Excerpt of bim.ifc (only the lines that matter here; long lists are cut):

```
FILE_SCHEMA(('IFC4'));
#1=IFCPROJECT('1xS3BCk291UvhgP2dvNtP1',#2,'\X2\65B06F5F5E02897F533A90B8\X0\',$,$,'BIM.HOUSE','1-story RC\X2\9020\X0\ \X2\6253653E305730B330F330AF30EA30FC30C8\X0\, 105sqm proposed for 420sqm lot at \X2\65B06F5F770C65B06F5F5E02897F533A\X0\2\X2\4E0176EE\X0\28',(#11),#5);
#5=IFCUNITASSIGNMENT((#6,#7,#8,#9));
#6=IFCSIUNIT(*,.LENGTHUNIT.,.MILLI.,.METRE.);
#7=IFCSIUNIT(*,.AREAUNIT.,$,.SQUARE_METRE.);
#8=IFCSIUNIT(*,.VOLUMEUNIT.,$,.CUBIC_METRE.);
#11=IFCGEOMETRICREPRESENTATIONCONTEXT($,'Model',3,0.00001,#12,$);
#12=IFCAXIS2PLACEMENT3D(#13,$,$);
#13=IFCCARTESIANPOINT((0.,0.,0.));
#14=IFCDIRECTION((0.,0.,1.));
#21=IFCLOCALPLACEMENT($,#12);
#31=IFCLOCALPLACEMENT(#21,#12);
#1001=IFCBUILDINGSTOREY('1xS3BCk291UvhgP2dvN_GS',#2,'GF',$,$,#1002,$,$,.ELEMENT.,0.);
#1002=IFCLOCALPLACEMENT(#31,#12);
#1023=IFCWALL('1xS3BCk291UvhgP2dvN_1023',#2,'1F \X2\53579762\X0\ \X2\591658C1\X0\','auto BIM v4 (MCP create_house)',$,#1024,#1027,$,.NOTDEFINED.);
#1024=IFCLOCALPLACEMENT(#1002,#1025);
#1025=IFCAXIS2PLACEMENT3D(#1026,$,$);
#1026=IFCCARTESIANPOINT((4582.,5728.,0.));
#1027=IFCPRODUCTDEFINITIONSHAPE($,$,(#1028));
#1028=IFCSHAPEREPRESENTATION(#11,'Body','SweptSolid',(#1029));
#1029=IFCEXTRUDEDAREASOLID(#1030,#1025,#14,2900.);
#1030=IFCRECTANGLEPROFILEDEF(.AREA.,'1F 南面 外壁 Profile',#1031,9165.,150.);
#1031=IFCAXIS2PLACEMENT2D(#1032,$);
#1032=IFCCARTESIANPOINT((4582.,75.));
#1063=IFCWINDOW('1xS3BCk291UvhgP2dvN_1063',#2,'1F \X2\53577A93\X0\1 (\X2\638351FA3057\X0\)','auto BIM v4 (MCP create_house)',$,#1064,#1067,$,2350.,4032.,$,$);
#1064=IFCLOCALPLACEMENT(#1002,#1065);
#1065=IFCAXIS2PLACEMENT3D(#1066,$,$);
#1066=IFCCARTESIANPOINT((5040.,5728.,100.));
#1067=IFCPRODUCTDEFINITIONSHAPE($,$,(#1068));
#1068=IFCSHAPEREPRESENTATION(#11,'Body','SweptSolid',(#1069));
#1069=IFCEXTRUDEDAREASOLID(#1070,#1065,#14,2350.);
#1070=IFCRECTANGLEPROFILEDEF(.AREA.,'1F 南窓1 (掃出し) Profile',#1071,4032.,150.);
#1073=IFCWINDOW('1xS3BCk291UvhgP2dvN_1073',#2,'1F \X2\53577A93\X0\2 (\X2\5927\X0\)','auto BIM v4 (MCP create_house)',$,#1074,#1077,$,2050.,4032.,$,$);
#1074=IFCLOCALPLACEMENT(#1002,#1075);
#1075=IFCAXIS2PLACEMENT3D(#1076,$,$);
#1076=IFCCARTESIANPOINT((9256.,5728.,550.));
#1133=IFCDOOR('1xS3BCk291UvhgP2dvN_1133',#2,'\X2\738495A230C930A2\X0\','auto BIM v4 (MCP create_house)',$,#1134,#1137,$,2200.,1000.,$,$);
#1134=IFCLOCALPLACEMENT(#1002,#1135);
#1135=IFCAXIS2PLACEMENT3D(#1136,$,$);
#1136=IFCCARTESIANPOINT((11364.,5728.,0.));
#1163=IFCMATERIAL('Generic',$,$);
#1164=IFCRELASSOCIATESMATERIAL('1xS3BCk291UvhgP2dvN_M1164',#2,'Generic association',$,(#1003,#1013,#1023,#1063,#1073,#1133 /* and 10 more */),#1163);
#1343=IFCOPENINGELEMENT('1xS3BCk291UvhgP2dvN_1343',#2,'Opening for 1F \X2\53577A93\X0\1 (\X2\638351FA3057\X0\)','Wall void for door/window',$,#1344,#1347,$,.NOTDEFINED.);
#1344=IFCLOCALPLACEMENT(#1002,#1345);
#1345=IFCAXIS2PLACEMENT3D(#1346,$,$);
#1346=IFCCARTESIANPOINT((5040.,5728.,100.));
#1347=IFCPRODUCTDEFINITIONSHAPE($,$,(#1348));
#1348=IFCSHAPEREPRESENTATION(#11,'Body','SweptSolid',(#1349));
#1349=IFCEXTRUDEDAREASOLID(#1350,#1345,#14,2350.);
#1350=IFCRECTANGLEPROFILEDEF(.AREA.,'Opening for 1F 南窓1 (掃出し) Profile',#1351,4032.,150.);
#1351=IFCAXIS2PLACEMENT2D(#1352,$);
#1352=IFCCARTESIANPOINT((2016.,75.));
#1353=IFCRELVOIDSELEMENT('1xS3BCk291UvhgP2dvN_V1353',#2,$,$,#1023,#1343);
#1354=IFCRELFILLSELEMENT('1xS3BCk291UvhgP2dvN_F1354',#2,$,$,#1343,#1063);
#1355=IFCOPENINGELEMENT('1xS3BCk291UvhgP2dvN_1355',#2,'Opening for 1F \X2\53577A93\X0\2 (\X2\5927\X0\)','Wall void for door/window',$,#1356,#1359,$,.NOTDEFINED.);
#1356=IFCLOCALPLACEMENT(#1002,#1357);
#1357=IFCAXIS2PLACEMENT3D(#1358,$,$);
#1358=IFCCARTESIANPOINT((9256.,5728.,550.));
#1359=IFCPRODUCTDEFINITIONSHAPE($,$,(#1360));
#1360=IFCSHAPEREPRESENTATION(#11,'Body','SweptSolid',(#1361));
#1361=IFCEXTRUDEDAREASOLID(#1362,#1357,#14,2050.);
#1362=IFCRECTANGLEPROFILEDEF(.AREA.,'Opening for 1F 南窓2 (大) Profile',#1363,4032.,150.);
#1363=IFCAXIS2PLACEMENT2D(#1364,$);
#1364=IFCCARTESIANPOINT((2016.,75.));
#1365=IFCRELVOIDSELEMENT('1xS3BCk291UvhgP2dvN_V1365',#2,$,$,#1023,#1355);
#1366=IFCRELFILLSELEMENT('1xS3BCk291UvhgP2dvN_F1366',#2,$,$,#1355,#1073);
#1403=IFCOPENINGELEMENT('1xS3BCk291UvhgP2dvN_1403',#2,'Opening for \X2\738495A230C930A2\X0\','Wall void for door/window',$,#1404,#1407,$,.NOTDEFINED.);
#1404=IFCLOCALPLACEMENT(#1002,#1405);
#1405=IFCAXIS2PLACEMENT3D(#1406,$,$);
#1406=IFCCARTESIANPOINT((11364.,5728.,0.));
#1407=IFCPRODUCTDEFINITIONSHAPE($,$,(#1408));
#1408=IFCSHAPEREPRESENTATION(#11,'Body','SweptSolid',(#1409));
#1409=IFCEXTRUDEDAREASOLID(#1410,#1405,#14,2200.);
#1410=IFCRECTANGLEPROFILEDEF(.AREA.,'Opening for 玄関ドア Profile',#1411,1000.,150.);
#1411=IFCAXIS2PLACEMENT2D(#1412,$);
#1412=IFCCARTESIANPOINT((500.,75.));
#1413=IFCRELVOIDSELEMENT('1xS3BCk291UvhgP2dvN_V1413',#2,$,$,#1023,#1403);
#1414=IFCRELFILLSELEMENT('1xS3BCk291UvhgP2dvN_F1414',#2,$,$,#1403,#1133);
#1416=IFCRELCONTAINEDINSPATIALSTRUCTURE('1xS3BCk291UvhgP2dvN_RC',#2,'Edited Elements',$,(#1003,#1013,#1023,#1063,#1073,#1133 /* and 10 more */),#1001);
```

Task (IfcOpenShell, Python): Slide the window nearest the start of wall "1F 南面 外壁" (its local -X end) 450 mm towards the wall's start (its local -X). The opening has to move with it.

```python
import ifcopenshell
import ifcopenshell.api.geometry
import ifcopenshell.util.placement

model = ifcopenshell.open("bim.ifc")

window = model.by_id(1063)
opening = window.FillsVoids[0].RelatingOpeningElement
wall = opening.VoidsElements[0].RelatingBuildingElement

wall_matrix = ifcopenshell.util.placement.get_local_placement(wall.ObjectPlacement)
shift = wall_matrix[:3, 0] * -450.0
before = ifcopenshell.util.placement.get_local_placement(window.ObjectPlacement)[:3, 3].copy()

# The window is not placed relative to its opening, so move both.
for product in (opening, window):
    matrix = ifcopenshell.util.placement.get_local_placement(product.ObjectPlacement)
    matrix[:3, 3] += shift
    ifcopenshell.api.geometry.edit_object_placement(model, product=product, matrix=matrix, is_si=False)

after = ifcopenshell.util.placement.get_local_placement(window.ObjectPlacement)[:3, 3]
print("window moved by", (after - before).round(3) + 0.0)

model.write("bim_rev.ifc")
```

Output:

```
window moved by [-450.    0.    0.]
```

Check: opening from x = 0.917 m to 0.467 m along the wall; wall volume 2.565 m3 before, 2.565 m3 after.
